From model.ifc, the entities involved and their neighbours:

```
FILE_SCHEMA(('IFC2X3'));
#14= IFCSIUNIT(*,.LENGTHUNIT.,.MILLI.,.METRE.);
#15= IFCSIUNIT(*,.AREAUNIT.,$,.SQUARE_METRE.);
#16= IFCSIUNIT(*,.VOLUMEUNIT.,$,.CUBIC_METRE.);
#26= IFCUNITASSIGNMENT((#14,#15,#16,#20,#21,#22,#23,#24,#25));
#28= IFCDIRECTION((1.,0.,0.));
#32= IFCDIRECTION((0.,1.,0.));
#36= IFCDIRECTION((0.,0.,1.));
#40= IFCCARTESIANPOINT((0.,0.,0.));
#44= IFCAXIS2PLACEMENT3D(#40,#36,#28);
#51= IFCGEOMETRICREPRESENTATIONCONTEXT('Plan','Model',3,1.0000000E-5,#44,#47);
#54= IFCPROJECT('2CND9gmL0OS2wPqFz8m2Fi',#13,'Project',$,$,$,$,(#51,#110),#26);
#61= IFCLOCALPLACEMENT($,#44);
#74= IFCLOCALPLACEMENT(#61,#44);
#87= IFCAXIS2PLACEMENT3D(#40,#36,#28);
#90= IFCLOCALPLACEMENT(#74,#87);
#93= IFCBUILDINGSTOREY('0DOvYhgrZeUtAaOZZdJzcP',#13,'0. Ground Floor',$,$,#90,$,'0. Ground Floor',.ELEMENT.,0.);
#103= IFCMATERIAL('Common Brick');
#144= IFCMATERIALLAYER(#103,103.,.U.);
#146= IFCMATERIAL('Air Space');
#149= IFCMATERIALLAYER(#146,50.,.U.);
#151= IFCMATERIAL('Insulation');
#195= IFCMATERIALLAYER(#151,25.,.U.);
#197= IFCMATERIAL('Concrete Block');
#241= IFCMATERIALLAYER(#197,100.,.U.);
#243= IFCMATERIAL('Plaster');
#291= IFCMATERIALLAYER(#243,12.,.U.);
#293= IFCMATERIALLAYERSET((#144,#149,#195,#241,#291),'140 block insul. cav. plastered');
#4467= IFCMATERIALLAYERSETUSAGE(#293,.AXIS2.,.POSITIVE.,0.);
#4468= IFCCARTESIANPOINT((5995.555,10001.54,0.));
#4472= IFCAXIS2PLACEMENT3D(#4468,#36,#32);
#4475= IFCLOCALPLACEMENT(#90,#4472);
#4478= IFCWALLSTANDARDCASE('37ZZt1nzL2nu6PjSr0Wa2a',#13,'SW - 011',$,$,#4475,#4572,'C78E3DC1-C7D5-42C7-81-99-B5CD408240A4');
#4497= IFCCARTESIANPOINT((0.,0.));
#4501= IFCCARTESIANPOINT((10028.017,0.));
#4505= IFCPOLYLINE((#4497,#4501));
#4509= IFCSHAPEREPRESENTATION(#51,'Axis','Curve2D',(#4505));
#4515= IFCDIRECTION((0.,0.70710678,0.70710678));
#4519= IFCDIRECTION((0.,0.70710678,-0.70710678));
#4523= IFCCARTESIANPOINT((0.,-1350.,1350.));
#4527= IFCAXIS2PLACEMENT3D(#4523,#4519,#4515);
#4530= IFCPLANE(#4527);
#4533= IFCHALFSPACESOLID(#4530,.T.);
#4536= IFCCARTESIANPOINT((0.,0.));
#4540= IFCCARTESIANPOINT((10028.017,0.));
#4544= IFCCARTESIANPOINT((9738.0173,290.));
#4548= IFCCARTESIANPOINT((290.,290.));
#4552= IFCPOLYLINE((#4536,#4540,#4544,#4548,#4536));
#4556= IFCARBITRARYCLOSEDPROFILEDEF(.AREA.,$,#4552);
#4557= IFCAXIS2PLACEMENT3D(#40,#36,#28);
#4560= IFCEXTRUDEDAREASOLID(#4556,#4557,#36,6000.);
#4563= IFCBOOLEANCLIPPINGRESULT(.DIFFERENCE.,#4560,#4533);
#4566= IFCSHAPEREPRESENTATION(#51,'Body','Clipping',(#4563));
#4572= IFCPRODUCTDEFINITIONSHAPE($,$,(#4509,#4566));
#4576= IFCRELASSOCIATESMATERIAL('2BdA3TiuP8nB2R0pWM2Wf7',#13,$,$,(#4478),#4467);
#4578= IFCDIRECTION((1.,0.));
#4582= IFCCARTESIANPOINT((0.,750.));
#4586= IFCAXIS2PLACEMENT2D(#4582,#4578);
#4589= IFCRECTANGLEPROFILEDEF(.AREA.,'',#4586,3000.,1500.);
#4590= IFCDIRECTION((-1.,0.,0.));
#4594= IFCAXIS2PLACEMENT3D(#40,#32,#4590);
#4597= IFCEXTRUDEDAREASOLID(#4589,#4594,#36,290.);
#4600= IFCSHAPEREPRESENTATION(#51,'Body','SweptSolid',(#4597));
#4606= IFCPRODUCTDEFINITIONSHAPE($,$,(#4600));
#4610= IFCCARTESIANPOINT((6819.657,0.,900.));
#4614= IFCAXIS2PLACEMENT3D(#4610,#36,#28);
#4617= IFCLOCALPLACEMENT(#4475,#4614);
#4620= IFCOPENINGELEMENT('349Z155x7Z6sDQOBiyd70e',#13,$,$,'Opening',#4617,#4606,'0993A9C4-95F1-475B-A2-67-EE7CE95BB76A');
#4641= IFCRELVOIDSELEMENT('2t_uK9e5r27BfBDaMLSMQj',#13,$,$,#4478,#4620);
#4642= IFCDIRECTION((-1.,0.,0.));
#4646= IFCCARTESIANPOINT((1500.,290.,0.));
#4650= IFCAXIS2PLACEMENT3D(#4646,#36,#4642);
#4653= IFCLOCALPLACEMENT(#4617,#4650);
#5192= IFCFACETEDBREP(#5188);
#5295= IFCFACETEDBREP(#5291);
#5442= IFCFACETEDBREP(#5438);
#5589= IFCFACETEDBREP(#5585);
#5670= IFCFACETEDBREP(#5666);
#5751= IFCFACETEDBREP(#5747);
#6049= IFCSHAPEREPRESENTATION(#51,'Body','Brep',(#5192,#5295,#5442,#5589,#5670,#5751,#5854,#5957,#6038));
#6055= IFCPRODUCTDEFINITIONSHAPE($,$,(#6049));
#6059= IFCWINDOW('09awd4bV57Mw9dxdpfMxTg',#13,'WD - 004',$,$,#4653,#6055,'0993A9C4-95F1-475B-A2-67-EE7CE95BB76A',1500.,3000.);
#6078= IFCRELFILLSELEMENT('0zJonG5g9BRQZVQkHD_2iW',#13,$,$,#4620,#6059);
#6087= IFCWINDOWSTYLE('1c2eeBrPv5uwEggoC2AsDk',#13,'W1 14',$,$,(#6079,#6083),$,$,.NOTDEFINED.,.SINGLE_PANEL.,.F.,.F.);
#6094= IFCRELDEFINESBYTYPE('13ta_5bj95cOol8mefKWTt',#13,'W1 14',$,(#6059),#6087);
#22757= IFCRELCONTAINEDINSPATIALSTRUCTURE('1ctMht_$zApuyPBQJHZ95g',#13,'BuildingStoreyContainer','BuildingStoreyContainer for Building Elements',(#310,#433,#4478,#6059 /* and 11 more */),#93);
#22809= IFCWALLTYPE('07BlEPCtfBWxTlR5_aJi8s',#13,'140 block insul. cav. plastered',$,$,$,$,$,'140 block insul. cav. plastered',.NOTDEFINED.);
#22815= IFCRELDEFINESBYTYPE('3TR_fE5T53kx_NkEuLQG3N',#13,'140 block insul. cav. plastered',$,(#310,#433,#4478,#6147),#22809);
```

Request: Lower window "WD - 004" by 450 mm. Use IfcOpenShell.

```python
import numpy as np
import ifcopenshell
import ifcopenshell.api.geometry
import ifcopenshell.util.placement
import ifcopenshell.util.unit

model = ifcopenshell.open("model.ifc")
unit_scale = ifcopenshell.util.unit.calculate_unit_scale(model)

window = model.by_id(6059)
opening = window.FillsVoids[0].RelatingOpeningElement
dz = -0.45 / unit_scale

shift = np.array([0.0, 0.0, dz])
# The window is placed relative to its opening, so it follows when the opening moves.
matrix = ifcopenshell.util.placement.get_local_placement(opening.ObjectPlacement)
matrix[:3, 3] += shift
ifcopenshell.api.geometry.edit_object_placement(
    model, product=opening, matrix=matrix, is_si=False, should_transform_children=True
)

print(f"moved by {dz * unit_scale:+.3f} m")

model.write("model_updated.ifc")
```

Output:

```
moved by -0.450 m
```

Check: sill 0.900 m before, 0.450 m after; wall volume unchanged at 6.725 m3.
